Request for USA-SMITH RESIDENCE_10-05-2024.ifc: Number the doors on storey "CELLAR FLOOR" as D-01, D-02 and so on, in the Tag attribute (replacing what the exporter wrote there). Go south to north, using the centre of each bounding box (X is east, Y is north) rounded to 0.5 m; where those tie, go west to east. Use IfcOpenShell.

First a look at what the model holds.

```python
import ifcopenshell
import ifcopenshell.util.element
import ifcopenshell.util.placement

model = ifcopenshell.open("USA-SMITH RESIDENCE_10-05-2024.ifc")
print(model.schema)
storey = next(s for s in model.by_type("IfcBuildingStorey") if s.Name == "CELLAR FLOOR")
doors = [e for e in ifcopenshell.util.element.get_decomposition(storey) if e.is_a("IfcDoor")]
for e in sorted(doors, key=lambda e: e.id()):
    origin = ifcopenshell.util.placement.get_local_placement(e.ObjectPlacement)[:3, 3]
    print(e.id(), e.Tag, e.Name, origin.round(2) + 0.0, sep=" | ")
```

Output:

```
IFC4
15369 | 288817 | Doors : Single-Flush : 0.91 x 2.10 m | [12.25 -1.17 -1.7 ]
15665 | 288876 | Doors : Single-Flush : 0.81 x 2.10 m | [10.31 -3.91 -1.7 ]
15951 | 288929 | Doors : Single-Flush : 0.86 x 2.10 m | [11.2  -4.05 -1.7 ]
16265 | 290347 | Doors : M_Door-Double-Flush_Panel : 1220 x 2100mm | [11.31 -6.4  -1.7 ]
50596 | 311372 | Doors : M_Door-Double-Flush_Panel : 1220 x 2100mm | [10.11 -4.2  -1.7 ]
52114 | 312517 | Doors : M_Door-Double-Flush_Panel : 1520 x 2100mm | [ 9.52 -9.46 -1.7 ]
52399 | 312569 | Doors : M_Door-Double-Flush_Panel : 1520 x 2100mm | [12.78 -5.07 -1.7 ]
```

```python
import ifcopenshell
import ifcopenshell.geom
import ifcopenshell.util.element
import ifcopenshell.util.shape

model = ifcopenshell.open("USA-SMITH RESIDENCE_10-05-2024.ifc")
settings = ifcopenshell.geom.settings()
settings.set("use-world-coords", True)


def centre(element):
    shape = ifcopenshell.geom.create_shape(settings, element)
    return ifcopenshell.util.shape.get_bbox_centroid(shape.geometry)


storey = next(s for s in model.by_type("IfcBuildingStorey") if s.Name == "CELLAR FLOOR")
doors = [e for e in ifcopenshell.util.element.get_decomposition(storey) if e.is_a("IfcDoor")]

# Insertion points can sit at a corner or the storey origin, so sort by the geometry (in metres).
centres = {e: centre(e) for e in doors}
doors.sort(key=lambda e: (round(centres[e][1] / 0.5), centres[e][0]))

for i, e in enumerate(doors, start=1):
    number = f"D-{i:02d}"
    e.Tag = number
    print(e.id(), number)

model.write("USA-SMITH RESIDENCE_10-05-2024_rev.ifc")
```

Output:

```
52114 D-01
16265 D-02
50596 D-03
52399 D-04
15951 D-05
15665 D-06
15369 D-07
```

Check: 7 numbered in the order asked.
